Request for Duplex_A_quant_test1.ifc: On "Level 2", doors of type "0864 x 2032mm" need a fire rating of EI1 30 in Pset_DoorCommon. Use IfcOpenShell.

First a look at what the model holds.

```python
import ifcopenshell
import ifcopenshell.util.element

model = ifcopenshell.open("Duplex_A_quant_test1.ifc")
print(model.schema)
storey = next(s for s in model.by_type("IfcBuildingStorey") if s.Name == "Level 2")
doors = [e for e in ifcopenshell.util.element.get_decomposition(storey) if e.is_a("IfcDoor")]
seen = {}
for e in doors:
    element_type = ifcopenshell.util.element.get_type(e)
    key = (element_type.Name if element_type != e and element_type else None, ifcopenshell.util.element.get_pset(e, "Pset_DoorCommon", "FireRating"))
    seen[key] = seen.get(key, 0) + 1
for (name, value), count in sorted(seen.items(), key=str):
    print(count, "x", name, "|", value)
```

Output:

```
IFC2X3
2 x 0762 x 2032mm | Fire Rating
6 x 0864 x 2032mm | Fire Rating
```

```python
import ifcopenshell
import ifcopenshell.api.pset
import ifcopenshell.util.element

model = ifcopenshell.open("Duplex_A_quant_test1.ifc")

storey = next(s for s in model.by_type("IfcBuildingStorey") if s.Name == "Level 2")
doors = [e for e in ifcopenshell.util.element.get_decomposition(storey) if e.is_a("IfcDoor")]

count = 0
for e in doors:
    element_type = ifcopenshell.util.element.get_type(e)
    if element_type in (None, e) or element_type.Name != "0864 x 2032mm":
        continue
    # add_pset returns the element's existing set when there is one.
    pset = ifcopenshell.api.pset.add_pset(model, product=e, name="Pset_DoorCommon")
    ifcopenshell.api.pset.edit_pset(model, pset=pset, properties={"FireRating": "EI1 30"})
    count += 1

print(count, "doors updated")

model.write("Duplex_A_quant_test1-out.ifc")
```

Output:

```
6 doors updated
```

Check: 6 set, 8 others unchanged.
